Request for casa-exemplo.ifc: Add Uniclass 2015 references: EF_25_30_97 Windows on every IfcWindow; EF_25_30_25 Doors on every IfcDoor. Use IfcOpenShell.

First a look at what the model holds.

```python
import ifcopenshell

model = ifcopenshell.open("casa-exemplo.ifc")
print(model.schema)
print("classifications:", [c.Name for c in model.by_type("IfcClassification")])
for ifc_class in ("IfcDoor", "IfcRoof", "IfcStair", "IfcWall", "IfcWindow"):
    print(ifc_class, len(model.by_type(ifc_class)))
```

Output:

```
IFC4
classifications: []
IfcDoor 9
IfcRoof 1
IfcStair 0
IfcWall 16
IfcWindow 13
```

```python
import ifcopenshell
import ifcopenshell.api.classification

model = ifcopenshell.open("casa-exemplo.ifc")

system = ifcopenshell.api.classification.add_classification(model, classification="Uniclass 2015")

codes = {
    "IfcWindow": ("EF_25_30_97", "Windows"),
    "IfcDoor": ("EF_25_30_25", "Doors"),
}
for ifc_class, (code, name) in codes.items():
    products = model.by_type(ifc_class)
    ifcopenshell.api.classification.add_reference(
        model, products=products, classification=system, identification=code, name=name
    )
    print(code, len(products))

model.write("casa-exemplo_updated.ifc")
```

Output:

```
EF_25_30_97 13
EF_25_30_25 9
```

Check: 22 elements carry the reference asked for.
